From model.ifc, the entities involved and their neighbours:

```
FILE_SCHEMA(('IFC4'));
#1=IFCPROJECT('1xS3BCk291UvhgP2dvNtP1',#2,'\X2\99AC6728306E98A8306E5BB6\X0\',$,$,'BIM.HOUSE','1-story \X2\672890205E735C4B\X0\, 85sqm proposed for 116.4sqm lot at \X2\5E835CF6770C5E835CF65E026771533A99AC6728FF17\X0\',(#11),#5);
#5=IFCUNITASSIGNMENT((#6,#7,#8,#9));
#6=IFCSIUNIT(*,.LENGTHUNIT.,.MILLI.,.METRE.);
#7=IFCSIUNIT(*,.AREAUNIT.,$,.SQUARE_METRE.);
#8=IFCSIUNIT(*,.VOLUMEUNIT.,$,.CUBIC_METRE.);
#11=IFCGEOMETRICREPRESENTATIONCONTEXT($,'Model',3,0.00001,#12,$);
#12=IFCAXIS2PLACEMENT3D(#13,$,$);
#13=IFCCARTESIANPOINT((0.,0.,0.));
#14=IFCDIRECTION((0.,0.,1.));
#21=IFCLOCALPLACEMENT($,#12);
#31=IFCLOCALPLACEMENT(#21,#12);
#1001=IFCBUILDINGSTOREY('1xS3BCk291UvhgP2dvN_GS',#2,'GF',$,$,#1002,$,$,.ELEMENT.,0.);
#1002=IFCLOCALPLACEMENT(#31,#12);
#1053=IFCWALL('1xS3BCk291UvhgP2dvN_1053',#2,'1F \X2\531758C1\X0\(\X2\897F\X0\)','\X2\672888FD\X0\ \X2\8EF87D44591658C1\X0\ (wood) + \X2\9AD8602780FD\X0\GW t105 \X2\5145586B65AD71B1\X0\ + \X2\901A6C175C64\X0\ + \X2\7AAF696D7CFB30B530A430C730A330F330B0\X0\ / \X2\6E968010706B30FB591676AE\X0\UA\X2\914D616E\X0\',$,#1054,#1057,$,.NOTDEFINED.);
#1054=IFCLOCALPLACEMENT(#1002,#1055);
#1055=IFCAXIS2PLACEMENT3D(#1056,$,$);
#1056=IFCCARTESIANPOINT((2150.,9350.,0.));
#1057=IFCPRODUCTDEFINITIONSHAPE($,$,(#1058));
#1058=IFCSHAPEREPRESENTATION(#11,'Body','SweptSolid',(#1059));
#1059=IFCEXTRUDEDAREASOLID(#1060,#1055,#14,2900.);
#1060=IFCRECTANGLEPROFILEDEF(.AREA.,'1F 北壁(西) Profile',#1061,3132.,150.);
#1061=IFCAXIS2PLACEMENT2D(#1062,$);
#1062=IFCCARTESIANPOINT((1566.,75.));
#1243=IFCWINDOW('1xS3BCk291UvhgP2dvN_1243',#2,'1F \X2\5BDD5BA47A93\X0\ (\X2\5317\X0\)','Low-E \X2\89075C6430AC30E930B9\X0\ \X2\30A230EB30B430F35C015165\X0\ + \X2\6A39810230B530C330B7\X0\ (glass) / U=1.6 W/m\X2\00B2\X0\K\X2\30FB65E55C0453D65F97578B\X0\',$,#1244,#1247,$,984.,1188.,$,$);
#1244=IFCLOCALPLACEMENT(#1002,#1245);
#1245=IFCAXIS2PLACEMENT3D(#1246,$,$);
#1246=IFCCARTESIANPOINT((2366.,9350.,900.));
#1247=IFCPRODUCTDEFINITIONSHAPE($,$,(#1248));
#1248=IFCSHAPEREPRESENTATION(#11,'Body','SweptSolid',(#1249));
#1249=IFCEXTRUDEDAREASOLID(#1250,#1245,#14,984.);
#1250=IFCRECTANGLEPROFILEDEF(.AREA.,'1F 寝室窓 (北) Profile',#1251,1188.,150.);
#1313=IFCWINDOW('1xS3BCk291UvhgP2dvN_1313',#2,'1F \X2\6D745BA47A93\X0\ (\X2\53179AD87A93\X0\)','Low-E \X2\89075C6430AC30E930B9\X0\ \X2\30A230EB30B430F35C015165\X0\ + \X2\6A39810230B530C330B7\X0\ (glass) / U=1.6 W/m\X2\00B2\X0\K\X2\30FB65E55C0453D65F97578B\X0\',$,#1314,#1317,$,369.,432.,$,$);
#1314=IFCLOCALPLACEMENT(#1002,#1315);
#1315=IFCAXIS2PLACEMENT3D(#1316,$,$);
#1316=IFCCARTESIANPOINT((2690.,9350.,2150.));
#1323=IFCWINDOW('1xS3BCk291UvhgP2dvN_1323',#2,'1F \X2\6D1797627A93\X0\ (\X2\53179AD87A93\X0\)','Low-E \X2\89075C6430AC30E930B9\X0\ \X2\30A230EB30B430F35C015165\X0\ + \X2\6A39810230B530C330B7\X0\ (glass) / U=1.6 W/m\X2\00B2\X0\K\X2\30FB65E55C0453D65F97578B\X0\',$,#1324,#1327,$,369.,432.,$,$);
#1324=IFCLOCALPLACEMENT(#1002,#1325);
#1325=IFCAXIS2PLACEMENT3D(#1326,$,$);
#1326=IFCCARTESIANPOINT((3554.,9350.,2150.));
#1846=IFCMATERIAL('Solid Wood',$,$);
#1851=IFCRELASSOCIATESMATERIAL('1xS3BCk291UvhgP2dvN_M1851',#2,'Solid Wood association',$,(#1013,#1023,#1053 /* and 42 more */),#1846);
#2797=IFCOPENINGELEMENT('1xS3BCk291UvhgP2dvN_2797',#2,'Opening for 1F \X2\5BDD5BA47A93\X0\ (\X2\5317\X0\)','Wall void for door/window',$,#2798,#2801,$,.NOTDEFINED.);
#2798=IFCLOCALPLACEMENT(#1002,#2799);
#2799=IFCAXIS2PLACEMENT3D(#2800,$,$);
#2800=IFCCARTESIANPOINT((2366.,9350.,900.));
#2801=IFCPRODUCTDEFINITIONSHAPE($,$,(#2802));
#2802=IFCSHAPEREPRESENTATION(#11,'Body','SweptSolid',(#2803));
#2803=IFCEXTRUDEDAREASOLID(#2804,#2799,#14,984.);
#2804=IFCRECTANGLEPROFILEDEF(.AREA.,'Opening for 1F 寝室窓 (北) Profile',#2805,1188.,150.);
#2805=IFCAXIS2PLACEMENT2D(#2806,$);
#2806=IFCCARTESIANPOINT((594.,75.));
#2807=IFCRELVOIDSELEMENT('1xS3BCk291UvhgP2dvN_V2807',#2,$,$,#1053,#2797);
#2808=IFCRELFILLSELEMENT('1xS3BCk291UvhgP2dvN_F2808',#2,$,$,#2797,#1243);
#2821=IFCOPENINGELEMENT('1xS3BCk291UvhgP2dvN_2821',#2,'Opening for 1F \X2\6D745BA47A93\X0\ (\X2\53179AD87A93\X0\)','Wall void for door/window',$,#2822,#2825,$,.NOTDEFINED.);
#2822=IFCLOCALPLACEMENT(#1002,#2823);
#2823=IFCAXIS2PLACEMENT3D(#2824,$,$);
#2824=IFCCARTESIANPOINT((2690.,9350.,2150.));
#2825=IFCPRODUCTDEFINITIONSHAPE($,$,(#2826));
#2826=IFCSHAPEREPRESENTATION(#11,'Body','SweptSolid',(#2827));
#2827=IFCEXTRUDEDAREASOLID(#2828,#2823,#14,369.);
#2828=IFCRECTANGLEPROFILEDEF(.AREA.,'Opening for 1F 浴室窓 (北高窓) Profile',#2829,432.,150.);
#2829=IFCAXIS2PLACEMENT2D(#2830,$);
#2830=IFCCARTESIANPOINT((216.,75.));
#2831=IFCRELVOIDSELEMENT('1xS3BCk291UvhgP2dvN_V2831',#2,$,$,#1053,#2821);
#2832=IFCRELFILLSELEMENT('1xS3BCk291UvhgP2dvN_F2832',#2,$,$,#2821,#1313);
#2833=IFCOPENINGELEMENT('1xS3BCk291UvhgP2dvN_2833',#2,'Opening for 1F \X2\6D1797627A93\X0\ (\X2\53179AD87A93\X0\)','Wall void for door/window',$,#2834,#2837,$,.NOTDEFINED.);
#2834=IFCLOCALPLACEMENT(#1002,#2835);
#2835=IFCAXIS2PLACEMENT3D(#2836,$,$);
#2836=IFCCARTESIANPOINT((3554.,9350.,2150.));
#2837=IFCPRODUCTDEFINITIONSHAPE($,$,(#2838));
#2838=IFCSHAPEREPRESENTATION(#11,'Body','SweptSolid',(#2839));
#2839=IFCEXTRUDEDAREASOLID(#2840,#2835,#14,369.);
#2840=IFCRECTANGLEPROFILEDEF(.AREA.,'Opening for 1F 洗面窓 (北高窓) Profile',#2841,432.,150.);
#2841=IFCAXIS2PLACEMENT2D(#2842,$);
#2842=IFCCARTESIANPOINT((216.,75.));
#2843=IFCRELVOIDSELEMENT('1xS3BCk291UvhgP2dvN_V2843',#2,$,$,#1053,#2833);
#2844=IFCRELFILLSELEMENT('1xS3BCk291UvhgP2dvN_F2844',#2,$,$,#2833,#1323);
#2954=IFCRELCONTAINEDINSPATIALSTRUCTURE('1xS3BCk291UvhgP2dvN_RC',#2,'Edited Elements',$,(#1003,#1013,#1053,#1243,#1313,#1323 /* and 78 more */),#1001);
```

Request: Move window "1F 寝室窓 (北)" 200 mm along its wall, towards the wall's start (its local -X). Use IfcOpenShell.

```python
import ifcopenshell
import ifcopenshell.api.geometry
import ifcopenshell.util.placement

model = ifcopenshell.open("model.ifc")

window = model.by_guid("1xS3BCk291UvhgP2dvN_1243")
opening = window.FillsVoids[0].RelatingOpeningElement
wall = opening.VoidsElements[0].RelatingBuildingElement

wall_matrix = ifcopenshell.util.placement.get_local_placement(wall.ObjectPlacement)
shift = wall_matrix[:3, 0] * -200.0
before = ifcopenshell.util.placement.get_local_placement(window.ObjectPlacement)[:3, 3].copy()

# The window is not placed relative to its opening, so move both.
for product in (opening, window):
    matrix = ifcopenshell.util.placement.get_local_placement(product.ObjectPlacement)
    matrix[:3, 3] += shift
    ifcopenshell.api.geometry.edit_object_placement(model, product=product, matrix=matrix, is_si=False)

after = ifcopenshell.util.placement.get_local_placement(window.ObjectPlacement)[:3, 3]
print("window moved by", (after - before).round(3) + 0.0)

model.write("model_edited.ifc")
```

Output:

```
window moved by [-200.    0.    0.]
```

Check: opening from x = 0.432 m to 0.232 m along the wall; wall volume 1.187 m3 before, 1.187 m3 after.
